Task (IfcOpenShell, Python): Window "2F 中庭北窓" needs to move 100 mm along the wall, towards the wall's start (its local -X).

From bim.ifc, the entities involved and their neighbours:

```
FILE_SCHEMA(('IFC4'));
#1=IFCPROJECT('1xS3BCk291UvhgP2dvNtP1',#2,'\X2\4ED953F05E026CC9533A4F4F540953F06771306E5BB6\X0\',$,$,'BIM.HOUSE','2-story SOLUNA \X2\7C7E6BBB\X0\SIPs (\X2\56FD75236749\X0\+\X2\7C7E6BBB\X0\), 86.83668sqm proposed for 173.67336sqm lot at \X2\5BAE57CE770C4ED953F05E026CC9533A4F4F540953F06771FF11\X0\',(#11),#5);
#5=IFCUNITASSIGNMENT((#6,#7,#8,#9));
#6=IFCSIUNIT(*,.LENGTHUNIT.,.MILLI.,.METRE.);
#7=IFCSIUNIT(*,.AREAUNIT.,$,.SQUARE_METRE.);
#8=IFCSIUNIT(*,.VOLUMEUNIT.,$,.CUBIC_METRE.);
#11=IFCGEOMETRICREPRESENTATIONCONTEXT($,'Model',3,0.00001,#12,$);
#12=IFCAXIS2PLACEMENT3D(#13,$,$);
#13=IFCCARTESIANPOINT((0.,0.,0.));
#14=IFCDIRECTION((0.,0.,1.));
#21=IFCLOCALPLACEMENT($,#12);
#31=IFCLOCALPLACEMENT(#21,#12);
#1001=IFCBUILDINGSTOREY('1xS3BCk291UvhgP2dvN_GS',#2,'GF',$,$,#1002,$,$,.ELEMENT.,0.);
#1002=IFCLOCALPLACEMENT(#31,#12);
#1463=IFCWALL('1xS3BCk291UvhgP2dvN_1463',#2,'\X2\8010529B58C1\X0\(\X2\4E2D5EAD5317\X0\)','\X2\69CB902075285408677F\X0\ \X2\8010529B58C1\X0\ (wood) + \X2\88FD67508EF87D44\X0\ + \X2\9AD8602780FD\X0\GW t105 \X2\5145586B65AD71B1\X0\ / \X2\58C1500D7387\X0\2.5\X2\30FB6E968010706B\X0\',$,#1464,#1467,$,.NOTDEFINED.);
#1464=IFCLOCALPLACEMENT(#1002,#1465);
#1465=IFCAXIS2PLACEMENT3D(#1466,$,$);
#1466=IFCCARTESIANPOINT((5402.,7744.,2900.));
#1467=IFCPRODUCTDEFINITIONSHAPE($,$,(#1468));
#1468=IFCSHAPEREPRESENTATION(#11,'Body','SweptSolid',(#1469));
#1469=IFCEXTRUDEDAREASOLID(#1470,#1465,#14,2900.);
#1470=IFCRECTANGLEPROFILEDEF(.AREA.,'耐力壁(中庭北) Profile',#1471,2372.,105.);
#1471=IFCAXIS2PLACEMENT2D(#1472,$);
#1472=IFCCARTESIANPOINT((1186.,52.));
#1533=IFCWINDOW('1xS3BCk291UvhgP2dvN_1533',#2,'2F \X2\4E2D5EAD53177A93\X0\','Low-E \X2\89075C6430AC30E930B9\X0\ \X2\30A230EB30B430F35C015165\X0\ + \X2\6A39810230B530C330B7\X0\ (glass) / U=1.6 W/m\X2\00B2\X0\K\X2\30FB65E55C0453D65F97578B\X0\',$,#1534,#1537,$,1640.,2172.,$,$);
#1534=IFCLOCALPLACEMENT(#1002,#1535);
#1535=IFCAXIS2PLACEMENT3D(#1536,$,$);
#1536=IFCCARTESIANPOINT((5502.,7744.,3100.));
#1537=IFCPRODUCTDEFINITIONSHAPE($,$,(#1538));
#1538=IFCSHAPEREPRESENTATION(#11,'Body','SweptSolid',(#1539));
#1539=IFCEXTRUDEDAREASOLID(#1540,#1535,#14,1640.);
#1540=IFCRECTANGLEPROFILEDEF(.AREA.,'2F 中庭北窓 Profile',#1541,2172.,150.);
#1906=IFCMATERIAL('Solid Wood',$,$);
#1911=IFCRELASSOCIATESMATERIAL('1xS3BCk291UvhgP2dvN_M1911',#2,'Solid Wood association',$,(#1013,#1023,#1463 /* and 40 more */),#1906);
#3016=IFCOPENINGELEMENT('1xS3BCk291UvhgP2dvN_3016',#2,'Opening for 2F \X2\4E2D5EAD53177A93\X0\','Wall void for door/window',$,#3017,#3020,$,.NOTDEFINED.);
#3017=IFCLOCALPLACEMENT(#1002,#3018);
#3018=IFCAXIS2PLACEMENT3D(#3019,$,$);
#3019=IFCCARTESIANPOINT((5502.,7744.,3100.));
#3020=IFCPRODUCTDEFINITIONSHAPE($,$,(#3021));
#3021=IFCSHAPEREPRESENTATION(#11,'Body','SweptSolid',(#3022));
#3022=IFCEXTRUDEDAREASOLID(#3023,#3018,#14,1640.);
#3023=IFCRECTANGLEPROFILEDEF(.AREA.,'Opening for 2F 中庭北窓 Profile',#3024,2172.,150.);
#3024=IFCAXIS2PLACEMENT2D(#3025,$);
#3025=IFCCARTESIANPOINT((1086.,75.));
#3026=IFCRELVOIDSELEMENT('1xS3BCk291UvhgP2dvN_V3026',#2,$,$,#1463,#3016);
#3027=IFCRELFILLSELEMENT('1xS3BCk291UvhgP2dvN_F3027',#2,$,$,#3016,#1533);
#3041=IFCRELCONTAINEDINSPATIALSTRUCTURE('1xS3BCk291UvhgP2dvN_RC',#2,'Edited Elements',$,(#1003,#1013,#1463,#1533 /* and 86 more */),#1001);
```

```python
import ifcopenshell
import ifcopenshell.api.geometry
import ifcopenshell.util.placement
import ifcopenshell.util.unit

model = ifcopenshell.open("bim.ifc")
unit_scale = ifcopenshell.util.unit.calculate_unit_scale(model)

window = model.by_guid("1xS3BCk291UvhgP2dvN_1533")
opening = window.FillsVoids[0].RelatingOpeningElement
wall = opening.VoidsElements[0].RelatingBuildingElement

wall_matrix = ifcopenshell.util.placement.get_local_placement(wall.ObjectPlacement)
shift = wall_matrix[:3, 0] * -0.1 / unit_scale
before = ifcopenshell.util.placement.get_local_placement(window.ObjectPlacement)[:3, 3].copy()

# The window is not placed relative to its opening, so move both.
for product in (opening, window):
    matrix = ifcopenshell.util.placement.get_local_placement(product.ObjectPlacement)
    matrix[:3, 3] += shift
    ifcopenshell.api.geometry.edit_object_placement(model, product=product, matrix=matrix, is_si=False)

after = ifcopenshell.util.placement.get_local_placement(window.ObjectPlacement)[:3, 3]
print("window moved by", (after - before).round(3) + 0.0)

model.write("bim_v2.ifc")
```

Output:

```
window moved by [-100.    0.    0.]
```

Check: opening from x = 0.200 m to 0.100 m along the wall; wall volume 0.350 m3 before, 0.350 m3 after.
